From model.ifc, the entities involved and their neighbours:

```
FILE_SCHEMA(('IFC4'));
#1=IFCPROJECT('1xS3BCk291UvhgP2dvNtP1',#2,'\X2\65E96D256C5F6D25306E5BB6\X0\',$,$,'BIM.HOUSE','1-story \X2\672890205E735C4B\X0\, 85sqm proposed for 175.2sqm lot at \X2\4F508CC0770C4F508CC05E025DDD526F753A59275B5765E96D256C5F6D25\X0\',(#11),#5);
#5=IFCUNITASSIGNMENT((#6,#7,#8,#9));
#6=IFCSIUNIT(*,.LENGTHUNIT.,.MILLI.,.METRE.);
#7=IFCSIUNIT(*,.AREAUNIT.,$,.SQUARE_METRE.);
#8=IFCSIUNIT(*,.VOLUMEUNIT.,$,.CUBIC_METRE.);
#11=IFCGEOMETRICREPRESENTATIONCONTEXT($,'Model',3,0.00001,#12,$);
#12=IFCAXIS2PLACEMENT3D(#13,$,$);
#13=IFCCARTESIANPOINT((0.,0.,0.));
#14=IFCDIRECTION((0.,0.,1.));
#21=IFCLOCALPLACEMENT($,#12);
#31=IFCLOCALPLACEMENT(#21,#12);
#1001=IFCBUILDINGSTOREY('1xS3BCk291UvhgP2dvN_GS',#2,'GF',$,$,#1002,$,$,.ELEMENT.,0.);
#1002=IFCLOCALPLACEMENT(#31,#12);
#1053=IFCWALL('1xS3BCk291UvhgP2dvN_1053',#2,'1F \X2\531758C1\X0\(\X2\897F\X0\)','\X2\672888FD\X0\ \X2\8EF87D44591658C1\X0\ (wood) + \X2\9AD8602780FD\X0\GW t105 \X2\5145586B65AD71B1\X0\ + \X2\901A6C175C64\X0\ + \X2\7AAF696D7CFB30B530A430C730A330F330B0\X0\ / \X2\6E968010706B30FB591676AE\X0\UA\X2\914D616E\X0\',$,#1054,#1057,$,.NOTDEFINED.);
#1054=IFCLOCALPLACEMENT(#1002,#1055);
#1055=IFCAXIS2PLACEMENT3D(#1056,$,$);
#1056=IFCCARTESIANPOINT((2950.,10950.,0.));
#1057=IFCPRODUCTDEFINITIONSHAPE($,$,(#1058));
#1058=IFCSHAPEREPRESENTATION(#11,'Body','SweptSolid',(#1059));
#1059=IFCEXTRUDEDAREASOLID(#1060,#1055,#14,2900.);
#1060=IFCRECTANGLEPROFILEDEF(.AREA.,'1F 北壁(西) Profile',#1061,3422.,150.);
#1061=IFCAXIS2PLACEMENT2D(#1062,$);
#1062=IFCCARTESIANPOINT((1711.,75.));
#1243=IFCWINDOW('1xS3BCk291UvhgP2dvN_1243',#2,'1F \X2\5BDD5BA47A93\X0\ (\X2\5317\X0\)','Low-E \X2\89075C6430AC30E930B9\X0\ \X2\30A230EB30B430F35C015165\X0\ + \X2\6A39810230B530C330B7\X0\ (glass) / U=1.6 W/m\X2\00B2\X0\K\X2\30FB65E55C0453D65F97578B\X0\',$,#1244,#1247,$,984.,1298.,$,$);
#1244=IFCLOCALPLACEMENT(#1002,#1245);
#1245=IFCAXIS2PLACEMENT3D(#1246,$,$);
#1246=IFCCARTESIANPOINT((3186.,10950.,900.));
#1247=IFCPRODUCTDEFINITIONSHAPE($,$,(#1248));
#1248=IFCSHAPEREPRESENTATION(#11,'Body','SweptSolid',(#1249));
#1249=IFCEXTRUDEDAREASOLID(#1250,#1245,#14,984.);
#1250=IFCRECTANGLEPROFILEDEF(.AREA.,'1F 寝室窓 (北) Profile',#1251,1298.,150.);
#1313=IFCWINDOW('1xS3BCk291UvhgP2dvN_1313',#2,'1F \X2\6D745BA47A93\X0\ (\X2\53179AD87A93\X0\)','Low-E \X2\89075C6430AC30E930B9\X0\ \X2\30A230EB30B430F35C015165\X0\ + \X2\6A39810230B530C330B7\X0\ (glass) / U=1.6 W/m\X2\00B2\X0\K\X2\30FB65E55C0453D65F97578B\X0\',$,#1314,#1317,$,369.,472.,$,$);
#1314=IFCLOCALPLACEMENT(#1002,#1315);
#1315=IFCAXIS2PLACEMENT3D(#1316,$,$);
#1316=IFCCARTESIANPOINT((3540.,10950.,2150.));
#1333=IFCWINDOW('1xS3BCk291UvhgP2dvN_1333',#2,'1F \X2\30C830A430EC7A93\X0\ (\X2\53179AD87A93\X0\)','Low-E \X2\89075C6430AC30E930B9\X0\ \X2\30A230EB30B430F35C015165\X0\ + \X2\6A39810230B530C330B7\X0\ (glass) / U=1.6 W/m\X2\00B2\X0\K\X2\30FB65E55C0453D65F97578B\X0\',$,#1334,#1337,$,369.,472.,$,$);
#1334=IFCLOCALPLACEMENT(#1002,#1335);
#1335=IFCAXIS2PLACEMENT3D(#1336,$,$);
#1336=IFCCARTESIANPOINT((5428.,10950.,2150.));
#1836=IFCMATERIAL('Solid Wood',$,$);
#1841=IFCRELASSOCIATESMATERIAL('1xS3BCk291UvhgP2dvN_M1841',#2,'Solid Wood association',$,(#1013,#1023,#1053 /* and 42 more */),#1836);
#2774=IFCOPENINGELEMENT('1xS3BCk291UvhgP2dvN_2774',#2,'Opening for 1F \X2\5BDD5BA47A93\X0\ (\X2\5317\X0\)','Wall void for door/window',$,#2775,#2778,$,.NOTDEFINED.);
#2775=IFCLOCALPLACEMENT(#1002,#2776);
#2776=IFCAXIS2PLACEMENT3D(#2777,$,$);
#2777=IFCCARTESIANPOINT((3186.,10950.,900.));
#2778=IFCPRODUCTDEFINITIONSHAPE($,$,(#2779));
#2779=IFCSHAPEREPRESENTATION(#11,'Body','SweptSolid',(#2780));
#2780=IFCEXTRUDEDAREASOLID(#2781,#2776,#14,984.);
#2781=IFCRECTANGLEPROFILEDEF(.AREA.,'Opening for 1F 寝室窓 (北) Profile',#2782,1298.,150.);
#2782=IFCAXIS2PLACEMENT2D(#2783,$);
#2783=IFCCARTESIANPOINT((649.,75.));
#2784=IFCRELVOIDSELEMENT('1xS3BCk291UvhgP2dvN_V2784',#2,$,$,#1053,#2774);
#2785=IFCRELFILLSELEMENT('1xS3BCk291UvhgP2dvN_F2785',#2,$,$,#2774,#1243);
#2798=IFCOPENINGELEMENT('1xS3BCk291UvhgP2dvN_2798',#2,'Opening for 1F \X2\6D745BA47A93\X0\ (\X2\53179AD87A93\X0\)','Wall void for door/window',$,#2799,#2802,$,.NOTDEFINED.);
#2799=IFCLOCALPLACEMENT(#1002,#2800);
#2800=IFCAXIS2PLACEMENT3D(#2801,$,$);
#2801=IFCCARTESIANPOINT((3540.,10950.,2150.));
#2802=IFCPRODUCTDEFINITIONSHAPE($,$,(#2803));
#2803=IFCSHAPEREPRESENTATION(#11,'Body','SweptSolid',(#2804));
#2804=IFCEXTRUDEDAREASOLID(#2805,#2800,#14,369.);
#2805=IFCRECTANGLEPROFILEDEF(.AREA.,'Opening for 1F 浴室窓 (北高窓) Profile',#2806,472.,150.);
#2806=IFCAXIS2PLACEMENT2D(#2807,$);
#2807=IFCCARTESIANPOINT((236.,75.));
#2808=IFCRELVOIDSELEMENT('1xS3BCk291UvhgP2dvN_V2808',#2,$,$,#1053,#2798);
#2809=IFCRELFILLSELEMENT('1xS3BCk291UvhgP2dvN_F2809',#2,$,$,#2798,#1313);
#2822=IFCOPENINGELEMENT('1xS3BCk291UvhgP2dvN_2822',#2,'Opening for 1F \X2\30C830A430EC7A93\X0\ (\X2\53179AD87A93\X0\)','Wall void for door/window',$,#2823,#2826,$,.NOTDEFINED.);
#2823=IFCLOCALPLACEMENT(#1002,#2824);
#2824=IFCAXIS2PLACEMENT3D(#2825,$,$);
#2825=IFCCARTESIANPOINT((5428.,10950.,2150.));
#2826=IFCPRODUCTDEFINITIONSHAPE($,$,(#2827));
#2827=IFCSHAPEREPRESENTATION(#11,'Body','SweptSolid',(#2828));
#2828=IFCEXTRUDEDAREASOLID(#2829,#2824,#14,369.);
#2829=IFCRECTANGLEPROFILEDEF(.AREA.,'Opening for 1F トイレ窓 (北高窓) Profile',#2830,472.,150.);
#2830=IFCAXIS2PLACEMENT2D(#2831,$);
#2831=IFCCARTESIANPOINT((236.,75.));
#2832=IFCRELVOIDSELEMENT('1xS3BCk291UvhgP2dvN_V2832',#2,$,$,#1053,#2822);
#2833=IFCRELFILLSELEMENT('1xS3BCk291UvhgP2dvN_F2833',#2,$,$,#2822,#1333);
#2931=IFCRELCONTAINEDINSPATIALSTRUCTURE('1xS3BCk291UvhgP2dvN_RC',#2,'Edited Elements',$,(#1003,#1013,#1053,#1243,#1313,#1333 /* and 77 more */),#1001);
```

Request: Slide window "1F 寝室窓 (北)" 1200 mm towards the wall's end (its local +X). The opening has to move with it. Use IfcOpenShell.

```python
import ifcopenshell
import ifcopenshell.api.geometry
import ifcopenshell.util.placement

model = ifcopenshell.open("model.ifc")

window = model.by_guid("1xS3BCk291UvhgP2dvN_1243")
opening = window.FillsVoids[0].RelatingOpeningElement
wall = opening.VoidsElements[0].RelatingBuildingElement

wall_matrix = ifcopenshell.util.placement.get_local_placement(wall.ObjectPlacement)
shift = wall_matrix[:3, 0] * 1200.0
before = ifcopenshell.util.placement.get_local_placement(window.ObjectPlacement)[:3, 3].copy()

# The window is not placed relative to its opening, so move both.
for product in (opening, window):
    matrix = ifcopenshell.util.placement.get_local_placement(product.ObjectPlacement)
    matrix[:3, 3] += shift
    ifcopenshell.api.geometry.edit_object_placement(model, product=product, matrix=matrix, is_si=False)

after = ifcopenshell.util.placement.get_local_placement(window.ObjectPlacement)[:3, 3]
print("window moved by", (after - before).round(3) + 0.0)

model.write("model_v2.ifc")
```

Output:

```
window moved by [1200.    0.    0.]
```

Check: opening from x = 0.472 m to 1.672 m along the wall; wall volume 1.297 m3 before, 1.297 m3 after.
